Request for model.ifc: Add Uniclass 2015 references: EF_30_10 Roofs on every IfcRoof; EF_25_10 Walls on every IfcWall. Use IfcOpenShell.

First a look at what the model holds.

```python
import ifcopenshell

model = ifcopenshell.open("model.ifc")
print(model.schema)
print("classifications:", [c.Name for c in model.by_type("IfcClassification")])
for ifc_class in ("IfcDoor", "IfcRoof", "IfcStair", "IfcWall", "IfcWindow"):
    print(ifc_class, len(model.by_type(ifc_class)))
```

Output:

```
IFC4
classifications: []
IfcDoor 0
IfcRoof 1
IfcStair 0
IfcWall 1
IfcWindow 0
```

```python
import ifcopenshell
import ifcopenshell.api.classification

model = ifcopenshell.open("model.ifc")

system = ifcopenshell.api.classification.add_classification(model, classification="Uniclass 2015")

codes = {
    "IfcRoof": ("EF_30_10", "Roofs"),
    "IfcWall": ("EF_25_10", "Walls"),
}
for ifc_class, (code, name) in codes.items():
    products = model.by_type(ifc_class)
    ifcopenshell.api.classification.add_reference(
        model, products=products, classification=system, identification=code, name=name
    )
    print(code, len(products))

model.write("model_updated.ifc")
```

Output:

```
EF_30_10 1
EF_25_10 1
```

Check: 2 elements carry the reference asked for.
